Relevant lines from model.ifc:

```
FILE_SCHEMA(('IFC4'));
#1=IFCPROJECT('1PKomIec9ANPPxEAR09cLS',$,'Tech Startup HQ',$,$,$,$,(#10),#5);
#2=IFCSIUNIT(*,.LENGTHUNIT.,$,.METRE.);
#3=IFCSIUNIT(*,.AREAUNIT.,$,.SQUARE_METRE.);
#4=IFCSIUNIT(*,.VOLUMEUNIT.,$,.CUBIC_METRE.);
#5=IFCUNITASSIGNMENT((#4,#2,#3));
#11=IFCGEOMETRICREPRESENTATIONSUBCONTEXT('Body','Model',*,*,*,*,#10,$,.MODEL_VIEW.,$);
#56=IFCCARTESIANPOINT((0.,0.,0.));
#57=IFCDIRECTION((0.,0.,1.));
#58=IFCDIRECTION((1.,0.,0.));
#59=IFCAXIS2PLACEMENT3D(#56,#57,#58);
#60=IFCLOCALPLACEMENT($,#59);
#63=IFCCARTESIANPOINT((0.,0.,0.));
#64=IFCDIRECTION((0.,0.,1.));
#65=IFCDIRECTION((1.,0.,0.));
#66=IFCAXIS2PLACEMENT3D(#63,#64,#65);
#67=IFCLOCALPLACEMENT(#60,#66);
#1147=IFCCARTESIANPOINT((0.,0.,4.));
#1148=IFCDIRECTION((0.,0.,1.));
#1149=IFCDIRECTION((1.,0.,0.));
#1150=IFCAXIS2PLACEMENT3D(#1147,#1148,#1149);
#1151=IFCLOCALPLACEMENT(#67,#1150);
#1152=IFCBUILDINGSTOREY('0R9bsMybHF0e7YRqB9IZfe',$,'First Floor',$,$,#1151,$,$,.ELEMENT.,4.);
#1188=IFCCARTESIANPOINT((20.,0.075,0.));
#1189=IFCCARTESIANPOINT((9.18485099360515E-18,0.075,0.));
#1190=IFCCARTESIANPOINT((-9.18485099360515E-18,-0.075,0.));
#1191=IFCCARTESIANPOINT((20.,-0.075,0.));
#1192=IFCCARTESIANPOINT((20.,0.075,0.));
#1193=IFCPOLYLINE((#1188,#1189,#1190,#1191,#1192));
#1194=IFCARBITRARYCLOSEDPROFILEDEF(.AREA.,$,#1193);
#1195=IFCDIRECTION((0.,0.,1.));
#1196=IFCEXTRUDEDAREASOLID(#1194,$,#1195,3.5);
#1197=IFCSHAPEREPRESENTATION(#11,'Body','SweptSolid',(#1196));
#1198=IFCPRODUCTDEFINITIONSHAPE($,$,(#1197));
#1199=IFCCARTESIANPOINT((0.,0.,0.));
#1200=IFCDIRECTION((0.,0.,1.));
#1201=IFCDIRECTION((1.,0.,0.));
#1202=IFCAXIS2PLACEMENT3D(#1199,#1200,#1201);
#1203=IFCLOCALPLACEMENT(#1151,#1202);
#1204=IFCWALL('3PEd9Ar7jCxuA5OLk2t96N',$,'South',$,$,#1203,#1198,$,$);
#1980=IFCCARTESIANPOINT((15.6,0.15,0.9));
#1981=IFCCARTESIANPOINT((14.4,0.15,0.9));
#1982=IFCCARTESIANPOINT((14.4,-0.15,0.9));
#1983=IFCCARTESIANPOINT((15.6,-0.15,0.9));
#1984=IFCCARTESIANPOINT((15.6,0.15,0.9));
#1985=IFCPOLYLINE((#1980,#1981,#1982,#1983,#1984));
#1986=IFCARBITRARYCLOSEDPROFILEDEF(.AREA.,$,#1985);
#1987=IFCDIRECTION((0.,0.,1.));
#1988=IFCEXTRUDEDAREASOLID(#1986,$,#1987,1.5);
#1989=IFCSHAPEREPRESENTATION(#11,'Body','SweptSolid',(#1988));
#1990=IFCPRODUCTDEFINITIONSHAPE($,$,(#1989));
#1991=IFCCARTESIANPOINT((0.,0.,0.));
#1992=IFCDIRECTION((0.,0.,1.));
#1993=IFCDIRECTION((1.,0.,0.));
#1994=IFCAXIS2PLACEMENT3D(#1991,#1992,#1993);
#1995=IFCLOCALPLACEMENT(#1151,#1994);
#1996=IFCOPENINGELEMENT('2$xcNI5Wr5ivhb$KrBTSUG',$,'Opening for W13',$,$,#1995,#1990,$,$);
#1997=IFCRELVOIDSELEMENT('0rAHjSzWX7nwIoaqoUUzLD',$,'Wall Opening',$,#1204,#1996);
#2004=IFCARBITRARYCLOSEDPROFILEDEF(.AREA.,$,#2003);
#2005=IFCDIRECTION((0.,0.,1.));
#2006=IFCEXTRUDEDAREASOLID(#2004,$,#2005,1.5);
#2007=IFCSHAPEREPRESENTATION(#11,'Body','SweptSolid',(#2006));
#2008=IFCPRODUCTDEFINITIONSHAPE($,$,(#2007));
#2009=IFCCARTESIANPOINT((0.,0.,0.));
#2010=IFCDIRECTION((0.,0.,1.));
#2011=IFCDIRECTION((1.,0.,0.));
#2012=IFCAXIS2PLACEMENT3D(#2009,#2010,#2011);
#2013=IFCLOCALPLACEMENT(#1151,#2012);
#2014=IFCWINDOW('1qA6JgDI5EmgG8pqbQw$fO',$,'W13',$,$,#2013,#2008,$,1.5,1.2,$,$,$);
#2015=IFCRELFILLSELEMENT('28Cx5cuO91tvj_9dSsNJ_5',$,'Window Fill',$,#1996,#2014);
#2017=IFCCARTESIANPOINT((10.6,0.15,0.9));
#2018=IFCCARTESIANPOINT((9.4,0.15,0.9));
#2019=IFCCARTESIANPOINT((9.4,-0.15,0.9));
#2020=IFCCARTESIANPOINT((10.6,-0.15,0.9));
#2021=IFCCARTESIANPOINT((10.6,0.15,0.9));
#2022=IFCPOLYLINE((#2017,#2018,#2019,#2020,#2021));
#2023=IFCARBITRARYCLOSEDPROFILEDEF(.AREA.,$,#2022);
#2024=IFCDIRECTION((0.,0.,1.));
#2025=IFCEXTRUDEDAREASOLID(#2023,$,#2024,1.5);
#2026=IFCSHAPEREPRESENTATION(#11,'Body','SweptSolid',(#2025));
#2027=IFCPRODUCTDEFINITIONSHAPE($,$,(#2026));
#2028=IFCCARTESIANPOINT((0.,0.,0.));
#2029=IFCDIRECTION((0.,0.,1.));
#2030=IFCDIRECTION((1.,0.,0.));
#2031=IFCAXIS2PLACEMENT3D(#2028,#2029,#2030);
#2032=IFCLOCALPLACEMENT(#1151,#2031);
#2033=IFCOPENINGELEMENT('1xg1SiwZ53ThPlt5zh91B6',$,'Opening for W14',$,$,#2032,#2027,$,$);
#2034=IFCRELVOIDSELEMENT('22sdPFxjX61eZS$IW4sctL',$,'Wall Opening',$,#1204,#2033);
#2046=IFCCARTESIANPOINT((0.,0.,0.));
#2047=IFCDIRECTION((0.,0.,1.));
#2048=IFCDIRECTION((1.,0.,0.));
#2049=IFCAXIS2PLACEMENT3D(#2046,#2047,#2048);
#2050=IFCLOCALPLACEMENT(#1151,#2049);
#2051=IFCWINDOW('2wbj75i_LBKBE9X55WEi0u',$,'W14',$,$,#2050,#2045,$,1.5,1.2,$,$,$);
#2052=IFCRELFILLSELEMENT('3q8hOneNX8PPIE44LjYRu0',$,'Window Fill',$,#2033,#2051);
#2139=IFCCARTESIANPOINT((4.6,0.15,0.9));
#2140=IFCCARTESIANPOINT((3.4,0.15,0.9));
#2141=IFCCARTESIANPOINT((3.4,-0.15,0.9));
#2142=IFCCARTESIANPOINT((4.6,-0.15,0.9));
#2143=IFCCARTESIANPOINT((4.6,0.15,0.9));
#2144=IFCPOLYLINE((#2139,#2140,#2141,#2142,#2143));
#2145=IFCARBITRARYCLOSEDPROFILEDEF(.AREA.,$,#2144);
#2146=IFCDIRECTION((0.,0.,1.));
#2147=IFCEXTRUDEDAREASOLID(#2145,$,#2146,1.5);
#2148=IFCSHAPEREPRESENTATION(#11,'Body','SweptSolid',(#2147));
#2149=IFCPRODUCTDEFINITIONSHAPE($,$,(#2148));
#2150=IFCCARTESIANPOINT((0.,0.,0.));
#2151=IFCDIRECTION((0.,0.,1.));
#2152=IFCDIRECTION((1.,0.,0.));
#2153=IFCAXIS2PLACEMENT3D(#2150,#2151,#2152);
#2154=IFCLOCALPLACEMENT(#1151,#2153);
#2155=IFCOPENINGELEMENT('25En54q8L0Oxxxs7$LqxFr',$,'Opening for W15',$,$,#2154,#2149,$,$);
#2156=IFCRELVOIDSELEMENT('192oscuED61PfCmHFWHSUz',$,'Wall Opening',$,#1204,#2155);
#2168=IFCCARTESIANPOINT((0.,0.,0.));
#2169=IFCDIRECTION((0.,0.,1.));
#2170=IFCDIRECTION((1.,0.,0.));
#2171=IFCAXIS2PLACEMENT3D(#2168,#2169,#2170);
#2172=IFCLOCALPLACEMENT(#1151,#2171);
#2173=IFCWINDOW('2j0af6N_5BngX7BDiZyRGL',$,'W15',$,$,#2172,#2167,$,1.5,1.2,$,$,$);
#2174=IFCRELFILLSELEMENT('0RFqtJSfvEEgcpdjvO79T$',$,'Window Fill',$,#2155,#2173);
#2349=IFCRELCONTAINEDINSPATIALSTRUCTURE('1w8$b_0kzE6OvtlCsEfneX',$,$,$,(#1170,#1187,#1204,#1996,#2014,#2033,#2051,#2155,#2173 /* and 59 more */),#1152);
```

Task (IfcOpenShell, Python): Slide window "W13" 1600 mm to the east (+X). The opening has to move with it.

```python
import ifcopenshell
import ifcopenshell.api.geometry
import ifcopenshell.util.placement
import ifcopenshell.util.unit

model = ifcopenshell.open("model.ifc")
unit_scale = ifcopenshell.util.unit.calculate_unit_scale(model)

window = model.by_guid("1qA6JgDI5EmgG8pqbQw$fO")
opening = window.FillsVoids[0].RelatingOpeningElement
wall = opening.VoidsElements[0].RelatingBuildingElement

wall_matrix = ifcopenshell.util.placement.get_local_placement(wall.ObjectPlacement)
shift = wall_matrix[:3, 0] * 1.6 / unit_scale
before = ifcopenshell.util.placement.get_local_placement(window.ObjectPlacement)[:3, 3].copy()

# The window is not placed relative to its opening, so move both.
for product in (opening, window):
    matrix = ifcopenshell.util.placement.get_local_placement(product.ObjectPlacement)
    matrix[:3, 3] += shift
    ifcopenshell.api.geometry.edit_object_placement(model, product=product, matrix=matrix, is_si=False)

after = ifcopenshell.util.placement.get_local_placement(window.ObjectPlacement)[:3, 3]
print("window moved by", (after - before).round(3) + 0.0)

model.write("model_edited.ifc")
```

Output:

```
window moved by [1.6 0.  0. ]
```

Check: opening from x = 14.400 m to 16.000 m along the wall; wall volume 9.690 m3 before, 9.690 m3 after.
